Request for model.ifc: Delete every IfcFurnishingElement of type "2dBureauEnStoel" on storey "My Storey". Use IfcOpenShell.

First a look at what the model holds.

```python
import ifcopenshell
import ifcopenshell.util.element

model = ifcopenshell.open("model.ifc")
print(model.schema)
storey = next(s for s in model.by_type("IfcBuildingStorey") if s.Name == "My Storey")
furniture = [e for e in ifcopenshell.util.element.get_decomposition(storey) if e.is_a("IfcFurnishingElement")]
seen = {}
for e in furniture:
    element_type = ifcopenshell.util.element.get_type(e)
    name = element_type.Name if element_type not in (None, e) else None
    seen[name] = seen.get(name, 0) + 1
for name, count in sorted(seen.items(), key=str):
    print(count, "x", name)
```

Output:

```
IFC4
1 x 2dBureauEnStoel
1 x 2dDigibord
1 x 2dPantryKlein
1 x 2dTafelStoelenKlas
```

```python
import ifcopenshell
import ifcopenshell.api.root
import ifcopenshell.util.element

model = ifcopenshell.open("model.ifc")

storey = next(s for s in model.by_type("IfcBuildingStorey") if s.Name == "My Storey")
furniture = [e for e in ifcopenshell.util.element.get_decomposition(storey) if e.is_a("IfcFurnishingElement")]
targets = [e for e in furniture if (t := ifcopenshell.util.element.get_type(e)) not in (None, e) and t.Name == "2dBureauEnStoel"]

for e in targets:
    ifcopenshell.api.root.remove_product(model, product=e)
print(len(targets), "removed")

model.write("model-out.ifc")
```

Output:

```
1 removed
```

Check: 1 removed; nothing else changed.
